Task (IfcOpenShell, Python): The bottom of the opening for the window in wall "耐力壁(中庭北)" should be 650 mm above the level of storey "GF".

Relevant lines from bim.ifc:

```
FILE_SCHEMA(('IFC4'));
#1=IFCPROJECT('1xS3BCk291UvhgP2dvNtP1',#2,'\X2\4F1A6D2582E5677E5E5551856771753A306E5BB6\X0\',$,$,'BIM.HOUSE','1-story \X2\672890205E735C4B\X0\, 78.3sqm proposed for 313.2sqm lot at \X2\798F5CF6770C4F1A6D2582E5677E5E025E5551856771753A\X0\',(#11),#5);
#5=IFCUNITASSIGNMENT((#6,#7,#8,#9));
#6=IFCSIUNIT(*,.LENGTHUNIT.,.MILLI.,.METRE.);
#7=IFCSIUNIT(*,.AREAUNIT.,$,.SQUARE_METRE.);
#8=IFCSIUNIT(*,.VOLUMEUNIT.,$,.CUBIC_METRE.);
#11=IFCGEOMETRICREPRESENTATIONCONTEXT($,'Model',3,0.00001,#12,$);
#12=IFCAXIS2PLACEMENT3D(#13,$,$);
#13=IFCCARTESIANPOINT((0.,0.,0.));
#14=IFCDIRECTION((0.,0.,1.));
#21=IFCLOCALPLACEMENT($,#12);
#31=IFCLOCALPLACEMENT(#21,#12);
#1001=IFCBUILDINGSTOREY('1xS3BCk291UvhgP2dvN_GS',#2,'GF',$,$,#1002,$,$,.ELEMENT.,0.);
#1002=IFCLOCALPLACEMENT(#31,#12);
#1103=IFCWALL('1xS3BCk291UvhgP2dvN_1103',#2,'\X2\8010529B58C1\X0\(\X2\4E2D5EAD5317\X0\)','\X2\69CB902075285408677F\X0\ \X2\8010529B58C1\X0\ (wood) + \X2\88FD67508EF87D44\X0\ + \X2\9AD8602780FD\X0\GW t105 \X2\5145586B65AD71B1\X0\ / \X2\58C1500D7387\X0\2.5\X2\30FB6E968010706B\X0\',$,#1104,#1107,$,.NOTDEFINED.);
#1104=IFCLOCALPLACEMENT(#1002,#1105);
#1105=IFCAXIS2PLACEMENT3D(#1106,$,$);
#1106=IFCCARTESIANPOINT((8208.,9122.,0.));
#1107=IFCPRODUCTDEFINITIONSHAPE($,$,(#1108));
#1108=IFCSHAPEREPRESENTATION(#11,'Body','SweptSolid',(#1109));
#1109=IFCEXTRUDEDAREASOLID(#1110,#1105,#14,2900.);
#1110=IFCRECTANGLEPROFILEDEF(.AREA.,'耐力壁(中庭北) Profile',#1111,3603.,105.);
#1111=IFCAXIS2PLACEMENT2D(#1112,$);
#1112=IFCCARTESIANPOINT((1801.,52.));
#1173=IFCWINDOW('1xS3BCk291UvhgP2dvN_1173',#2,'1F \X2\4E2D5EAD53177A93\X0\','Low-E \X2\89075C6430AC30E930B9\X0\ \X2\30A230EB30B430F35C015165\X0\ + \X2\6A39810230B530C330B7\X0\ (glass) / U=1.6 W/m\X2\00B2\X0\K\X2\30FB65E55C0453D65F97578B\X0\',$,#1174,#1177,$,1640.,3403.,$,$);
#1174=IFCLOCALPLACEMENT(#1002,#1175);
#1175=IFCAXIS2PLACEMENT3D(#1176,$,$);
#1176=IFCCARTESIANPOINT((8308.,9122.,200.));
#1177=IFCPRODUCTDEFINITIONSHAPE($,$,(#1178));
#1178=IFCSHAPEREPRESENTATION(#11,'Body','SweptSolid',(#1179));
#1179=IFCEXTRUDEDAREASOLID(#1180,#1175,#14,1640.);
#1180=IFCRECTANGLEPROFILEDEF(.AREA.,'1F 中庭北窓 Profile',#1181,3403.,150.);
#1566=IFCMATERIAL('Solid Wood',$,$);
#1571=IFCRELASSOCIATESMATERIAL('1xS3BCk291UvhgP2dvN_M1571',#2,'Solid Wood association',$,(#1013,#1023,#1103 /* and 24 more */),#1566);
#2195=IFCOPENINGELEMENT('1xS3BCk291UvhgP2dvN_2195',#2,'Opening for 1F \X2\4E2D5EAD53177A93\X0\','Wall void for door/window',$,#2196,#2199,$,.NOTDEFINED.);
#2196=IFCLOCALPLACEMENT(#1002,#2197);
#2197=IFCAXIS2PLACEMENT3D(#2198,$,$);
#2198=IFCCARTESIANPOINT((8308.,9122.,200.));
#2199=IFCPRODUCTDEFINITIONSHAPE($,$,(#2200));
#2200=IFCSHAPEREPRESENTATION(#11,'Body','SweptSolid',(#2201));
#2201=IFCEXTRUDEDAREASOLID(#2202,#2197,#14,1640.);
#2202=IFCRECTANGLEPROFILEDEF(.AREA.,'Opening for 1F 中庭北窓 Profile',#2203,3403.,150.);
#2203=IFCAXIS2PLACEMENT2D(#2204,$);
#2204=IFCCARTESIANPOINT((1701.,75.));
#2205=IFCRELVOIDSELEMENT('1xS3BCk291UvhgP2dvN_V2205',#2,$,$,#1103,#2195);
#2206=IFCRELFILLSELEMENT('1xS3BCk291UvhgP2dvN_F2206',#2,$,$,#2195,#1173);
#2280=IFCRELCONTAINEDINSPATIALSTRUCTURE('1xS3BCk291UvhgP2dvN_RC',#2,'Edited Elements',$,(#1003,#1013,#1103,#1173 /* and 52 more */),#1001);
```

```python
import numpy as np
import ifcopenshell
import ifcopenshell.api.geometry
import ifcopenshell.geom
import ifcopenshell.util.element
import ifcopenshell.util.placement
import ifcopenshell.util.shape
import ifcopenshell.util.unit

model = ifcopenshell.open("bim.ifc")
unit_scale = ifcopenshell.util.unit.calculate_unit_scale(model)

window = model.by_guid("1xS3BCk291UvhgP2dvN_1173")
opening = window.FillsVoids[0].RelatingOpeningElement
storey = ifcopenshell.util.element.get_container(window, ifc_class="IfcBuildingStorey")
level = ifcopenshell.util.placement.get_local_placement(storey.ObjectPlacement)[2, 3]

# The opening's origin need not be at the sill, so measure its lowest point.
shape = ifcopenshell.geom.create_shape(ifcopenshell.geom.settings(), opening)
bottom = ifcopenshell.util.shape.get_shape_bottom_elevation(shape, shape.geometry) / unit_scale
dz = level + 0.65 / unit_scale - bottom

shift = np.array([0.0, 0.0, dz])
# The window is not placed relative to its opening, so move both.
for product in (opening, window):
    matrix = ifcopenshell.util.placement.get_local_placement(product.ObjectPlacement)
    matrix[:3, 3] += shift
    ifcopenshell.api.geometry.edit_object_placement(model, product=product, matrix=matrix, is_si=False)

print(f"moved by {dz * unit_scale:+.3f} m")

model.write("bim_updated.ifc")
```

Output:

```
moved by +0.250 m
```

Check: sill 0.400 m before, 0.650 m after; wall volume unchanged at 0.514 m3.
